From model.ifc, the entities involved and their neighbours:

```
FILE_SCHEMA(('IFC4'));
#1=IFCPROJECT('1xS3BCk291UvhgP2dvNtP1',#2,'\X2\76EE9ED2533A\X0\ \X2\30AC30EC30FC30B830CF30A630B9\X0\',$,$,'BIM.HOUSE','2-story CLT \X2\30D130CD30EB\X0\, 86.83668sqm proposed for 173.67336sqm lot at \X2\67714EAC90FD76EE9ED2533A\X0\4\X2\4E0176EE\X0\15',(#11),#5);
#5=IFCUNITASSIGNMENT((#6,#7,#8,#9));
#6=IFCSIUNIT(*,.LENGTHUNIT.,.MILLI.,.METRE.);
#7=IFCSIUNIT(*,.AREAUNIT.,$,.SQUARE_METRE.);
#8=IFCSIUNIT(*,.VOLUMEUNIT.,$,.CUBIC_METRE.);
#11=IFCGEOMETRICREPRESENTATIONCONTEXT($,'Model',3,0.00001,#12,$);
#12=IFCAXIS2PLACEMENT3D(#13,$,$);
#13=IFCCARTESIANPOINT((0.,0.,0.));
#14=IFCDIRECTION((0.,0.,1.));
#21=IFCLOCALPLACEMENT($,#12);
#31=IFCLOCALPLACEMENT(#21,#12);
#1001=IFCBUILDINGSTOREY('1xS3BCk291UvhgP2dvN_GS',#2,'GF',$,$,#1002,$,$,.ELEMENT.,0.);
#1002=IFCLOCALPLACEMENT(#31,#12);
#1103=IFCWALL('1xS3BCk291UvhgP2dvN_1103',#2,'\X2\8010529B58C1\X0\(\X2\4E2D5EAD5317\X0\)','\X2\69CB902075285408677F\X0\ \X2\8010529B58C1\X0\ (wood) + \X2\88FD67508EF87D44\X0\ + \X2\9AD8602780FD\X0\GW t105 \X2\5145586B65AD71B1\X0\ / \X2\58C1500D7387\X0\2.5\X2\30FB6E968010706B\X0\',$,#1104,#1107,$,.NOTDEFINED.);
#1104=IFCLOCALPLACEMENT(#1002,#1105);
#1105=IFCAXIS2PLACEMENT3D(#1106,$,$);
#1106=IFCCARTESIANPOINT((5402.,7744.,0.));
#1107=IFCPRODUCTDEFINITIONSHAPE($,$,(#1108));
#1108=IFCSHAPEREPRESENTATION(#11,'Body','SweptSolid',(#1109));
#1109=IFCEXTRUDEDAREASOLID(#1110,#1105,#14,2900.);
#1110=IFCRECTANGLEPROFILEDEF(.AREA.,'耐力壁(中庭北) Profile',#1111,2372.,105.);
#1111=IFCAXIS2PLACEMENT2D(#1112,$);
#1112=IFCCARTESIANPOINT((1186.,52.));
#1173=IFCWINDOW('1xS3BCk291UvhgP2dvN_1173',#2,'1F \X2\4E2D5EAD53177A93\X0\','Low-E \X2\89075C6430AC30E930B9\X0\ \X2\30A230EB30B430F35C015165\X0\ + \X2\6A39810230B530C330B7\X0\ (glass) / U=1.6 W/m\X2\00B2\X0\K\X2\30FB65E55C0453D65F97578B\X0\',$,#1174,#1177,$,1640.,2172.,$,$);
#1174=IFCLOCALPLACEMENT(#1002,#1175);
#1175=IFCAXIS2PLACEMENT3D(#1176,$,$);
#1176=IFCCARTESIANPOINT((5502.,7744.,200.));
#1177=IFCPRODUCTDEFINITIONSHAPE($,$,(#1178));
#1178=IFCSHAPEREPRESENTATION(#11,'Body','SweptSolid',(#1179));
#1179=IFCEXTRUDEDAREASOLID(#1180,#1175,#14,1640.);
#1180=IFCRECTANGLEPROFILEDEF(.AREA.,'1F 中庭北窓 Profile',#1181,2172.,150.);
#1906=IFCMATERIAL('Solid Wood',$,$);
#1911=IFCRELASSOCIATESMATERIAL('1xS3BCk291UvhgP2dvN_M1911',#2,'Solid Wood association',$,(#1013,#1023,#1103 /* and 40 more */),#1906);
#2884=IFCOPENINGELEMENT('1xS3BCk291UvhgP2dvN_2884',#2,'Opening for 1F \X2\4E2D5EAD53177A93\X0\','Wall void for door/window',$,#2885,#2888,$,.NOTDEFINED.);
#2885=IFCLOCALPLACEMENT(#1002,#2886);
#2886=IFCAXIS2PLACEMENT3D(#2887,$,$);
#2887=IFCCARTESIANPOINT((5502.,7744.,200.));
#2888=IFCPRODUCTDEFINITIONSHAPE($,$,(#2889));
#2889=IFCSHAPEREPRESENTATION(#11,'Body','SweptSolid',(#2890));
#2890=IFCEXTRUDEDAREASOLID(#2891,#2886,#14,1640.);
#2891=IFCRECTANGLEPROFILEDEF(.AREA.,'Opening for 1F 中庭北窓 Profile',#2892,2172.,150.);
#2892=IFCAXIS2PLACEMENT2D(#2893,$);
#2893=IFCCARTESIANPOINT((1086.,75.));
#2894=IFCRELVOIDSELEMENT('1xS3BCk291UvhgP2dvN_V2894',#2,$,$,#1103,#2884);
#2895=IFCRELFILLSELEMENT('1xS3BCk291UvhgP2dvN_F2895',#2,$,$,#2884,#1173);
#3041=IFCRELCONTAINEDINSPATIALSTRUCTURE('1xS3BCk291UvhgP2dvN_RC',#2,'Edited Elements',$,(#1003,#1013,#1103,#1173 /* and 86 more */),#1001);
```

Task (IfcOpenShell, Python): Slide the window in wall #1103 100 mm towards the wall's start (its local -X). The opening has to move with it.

```python
import ifcopenshell
import ifcopenshell.api.geometry
import ifcopenshell.util.placement
import ifcopenshell.util.unit

model = ifcopenshell.open("model.ifc")
unit_scale = ifcopenshell.util.unit.calculate_unit_scale(model)

window = model.by_guid("1xS3BCk291UvhgP2dvN_1173")
opening = window.FillsVoids[0].RelatingOpeningElement
wall = opening.VoidsElements[0].RelatingBuildingElement

wall_matrix = ifcopenshell.util.placement.get_local_placement(wall.ObjectPlacement)
shift = wall_matrix[:3, 0] * -0.1 / unit_scale
before = ifcopenshell.util.placement.get_local_placement(window.ObjectPlacement)[:3, 3].copy()

# The window is not placed relative to its opening, so move both.
for product in (opening, window):
    matrix = ifcopenshell.util.placement.get_local_placement(product.ObjectPlacement)
    matrix[:3, 3] += shift
    ifcopenshell.api.geometry.edit_object_placement(model, product=product, matrix=matrix, is_si=False)

after = ifcopenshell.util.placement.get_local_placement(window.ObjectPlacement)[:3, 3]
print("window moved by", (after - before).round(3) + 0.0)

model.write("model-out.ifc")
```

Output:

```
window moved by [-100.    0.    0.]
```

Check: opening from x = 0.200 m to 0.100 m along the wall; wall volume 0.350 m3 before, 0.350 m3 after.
